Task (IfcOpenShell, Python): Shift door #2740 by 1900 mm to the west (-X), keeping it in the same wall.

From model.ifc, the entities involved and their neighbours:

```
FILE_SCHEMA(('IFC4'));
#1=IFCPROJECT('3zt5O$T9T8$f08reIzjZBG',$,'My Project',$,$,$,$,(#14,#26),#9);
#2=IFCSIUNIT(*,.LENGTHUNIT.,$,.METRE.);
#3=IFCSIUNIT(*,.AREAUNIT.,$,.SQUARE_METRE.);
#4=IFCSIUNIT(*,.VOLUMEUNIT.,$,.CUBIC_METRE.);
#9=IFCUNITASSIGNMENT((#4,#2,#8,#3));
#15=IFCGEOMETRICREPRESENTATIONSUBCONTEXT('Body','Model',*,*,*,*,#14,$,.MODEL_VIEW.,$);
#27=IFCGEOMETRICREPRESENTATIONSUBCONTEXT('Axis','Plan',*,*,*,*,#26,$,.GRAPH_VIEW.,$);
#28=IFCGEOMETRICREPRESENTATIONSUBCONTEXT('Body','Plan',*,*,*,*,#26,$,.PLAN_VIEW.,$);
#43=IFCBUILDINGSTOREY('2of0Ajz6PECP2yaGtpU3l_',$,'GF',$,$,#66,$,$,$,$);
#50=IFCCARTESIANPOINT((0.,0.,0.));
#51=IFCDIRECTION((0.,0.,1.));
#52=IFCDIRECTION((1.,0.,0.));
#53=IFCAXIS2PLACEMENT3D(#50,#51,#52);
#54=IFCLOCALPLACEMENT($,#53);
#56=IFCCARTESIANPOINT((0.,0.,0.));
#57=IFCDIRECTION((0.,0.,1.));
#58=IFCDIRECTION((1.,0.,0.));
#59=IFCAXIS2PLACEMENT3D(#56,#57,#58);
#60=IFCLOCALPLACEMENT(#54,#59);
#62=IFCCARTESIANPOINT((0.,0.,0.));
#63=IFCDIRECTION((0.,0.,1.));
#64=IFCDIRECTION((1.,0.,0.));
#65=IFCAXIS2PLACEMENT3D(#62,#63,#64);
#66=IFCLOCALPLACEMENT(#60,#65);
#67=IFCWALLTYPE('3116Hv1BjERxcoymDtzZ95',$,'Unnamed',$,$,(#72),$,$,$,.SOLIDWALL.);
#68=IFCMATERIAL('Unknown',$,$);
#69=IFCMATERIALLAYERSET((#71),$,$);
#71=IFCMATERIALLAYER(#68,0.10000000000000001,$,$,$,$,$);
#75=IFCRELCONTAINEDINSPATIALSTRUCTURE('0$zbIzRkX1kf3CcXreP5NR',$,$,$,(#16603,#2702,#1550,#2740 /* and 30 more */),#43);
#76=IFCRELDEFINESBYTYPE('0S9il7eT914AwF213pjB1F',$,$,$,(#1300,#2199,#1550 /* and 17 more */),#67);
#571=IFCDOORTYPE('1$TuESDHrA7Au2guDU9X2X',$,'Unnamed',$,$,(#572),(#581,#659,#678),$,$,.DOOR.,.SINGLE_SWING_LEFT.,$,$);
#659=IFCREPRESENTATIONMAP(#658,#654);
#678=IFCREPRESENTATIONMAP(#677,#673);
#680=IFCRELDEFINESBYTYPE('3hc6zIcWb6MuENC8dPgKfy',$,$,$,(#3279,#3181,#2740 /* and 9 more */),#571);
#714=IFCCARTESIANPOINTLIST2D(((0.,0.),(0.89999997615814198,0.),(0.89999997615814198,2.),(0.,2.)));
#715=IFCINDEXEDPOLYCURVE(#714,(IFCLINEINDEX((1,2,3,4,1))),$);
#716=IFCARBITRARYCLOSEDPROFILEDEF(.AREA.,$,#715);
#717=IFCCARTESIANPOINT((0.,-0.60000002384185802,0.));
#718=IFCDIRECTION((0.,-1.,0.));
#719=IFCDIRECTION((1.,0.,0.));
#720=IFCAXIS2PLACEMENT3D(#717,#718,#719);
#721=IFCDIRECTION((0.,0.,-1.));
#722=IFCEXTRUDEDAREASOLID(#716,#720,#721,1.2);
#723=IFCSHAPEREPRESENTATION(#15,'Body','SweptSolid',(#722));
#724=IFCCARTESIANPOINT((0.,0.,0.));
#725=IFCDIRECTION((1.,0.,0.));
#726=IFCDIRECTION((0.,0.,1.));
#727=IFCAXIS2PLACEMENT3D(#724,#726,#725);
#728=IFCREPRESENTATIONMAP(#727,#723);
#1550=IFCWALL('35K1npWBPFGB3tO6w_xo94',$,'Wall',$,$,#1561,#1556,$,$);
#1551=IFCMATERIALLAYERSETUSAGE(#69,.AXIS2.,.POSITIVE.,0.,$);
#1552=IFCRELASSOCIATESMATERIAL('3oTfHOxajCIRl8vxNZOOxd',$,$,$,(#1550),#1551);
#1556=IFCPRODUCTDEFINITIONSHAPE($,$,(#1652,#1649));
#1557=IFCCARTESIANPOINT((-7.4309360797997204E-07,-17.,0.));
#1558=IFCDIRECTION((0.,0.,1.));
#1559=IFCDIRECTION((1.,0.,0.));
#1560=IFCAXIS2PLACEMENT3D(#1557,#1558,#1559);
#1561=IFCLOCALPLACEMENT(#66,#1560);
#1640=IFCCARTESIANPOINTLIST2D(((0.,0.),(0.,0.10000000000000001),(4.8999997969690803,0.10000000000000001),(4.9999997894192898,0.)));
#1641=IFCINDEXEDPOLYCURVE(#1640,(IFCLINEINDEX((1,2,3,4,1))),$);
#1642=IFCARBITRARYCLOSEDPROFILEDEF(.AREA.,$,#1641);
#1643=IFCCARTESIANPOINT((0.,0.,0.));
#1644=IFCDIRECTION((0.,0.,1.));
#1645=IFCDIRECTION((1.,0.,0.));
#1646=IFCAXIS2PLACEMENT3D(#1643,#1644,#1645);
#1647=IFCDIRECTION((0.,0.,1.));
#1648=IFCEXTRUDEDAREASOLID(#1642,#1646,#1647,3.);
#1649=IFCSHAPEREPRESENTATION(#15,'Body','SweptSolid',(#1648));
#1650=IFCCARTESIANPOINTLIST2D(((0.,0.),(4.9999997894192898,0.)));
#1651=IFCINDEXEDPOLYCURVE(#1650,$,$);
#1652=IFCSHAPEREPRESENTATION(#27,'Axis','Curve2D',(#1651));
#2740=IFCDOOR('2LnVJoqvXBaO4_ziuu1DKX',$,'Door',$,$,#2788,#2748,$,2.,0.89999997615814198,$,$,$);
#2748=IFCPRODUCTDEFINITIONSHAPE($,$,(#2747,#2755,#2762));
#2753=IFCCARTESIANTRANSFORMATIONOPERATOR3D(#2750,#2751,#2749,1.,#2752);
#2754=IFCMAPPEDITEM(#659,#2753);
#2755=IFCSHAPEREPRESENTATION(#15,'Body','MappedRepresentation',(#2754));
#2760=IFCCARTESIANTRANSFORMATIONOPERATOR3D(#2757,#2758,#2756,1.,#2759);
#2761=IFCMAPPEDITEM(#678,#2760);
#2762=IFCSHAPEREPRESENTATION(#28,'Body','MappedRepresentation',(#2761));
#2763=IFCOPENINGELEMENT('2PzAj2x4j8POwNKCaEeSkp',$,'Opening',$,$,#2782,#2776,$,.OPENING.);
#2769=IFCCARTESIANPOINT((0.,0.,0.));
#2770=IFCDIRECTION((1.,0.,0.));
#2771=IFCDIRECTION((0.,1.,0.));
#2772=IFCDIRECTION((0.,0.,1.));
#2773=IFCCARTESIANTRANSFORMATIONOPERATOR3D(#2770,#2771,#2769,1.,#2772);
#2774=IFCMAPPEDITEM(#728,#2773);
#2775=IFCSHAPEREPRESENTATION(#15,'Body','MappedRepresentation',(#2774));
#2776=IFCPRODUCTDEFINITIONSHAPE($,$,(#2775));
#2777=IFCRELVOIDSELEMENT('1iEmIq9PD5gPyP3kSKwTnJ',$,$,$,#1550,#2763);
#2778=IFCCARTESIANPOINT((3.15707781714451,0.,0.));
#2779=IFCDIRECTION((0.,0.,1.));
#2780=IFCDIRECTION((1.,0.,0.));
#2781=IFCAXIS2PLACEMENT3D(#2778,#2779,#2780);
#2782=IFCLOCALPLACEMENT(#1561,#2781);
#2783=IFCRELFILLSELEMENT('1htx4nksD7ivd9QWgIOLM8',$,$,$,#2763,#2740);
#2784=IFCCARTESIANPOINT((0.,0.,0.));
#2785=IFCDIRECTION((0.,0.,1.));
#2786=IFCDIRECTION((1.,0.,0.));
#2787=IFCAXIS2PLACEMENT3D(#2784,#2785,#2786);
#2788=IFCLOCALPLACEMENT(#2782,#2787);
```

```python
import ifcopenshell
import ifcopenshell.api.geometry
import ifcopenshell.util.placement

model = ifcopenshell.open("model.ifc")

door = model.by_guid("2LnVJoqvXBaO4_ziuu1DKX")
opening = door.FillsVoids[0].RelatingOpeningElement
wall = opening.VoidsElements[0].RelatingBuildingElement

wall_matrix = ifcopenshell.util.placement.get_local_placement(wall.ObjectPlacement)
shift = wall_matrix[:3, 0] * -1.9
before = ifcopenshell.util.placement.get_local_placement(door.ObjectPlacement)[:3, 3].copy()

# The door is placed relative to its opening, so it follows when the opening moves.
matrix = ifcopenshell.util.placement.get_local_placement(opening.ObjectPlacement)
matrix[:3, 3] += shift
ifcopenshell.api.geometry.edit_object_placement(
    model, product=opening, matrix=matrix, is_si=False, should_transform_children=True
)

after = ifcopenshell.util.placement.get_local_placement(door.ObjectPlacement)[:3, 3]
print("door moved by", (after - before).round(3) + 0.0)

model.write("model_v2.ifc")
```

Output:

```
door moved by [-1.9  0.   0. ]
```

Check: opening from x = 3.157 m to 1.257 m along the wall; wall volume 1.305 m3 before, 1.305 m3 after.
